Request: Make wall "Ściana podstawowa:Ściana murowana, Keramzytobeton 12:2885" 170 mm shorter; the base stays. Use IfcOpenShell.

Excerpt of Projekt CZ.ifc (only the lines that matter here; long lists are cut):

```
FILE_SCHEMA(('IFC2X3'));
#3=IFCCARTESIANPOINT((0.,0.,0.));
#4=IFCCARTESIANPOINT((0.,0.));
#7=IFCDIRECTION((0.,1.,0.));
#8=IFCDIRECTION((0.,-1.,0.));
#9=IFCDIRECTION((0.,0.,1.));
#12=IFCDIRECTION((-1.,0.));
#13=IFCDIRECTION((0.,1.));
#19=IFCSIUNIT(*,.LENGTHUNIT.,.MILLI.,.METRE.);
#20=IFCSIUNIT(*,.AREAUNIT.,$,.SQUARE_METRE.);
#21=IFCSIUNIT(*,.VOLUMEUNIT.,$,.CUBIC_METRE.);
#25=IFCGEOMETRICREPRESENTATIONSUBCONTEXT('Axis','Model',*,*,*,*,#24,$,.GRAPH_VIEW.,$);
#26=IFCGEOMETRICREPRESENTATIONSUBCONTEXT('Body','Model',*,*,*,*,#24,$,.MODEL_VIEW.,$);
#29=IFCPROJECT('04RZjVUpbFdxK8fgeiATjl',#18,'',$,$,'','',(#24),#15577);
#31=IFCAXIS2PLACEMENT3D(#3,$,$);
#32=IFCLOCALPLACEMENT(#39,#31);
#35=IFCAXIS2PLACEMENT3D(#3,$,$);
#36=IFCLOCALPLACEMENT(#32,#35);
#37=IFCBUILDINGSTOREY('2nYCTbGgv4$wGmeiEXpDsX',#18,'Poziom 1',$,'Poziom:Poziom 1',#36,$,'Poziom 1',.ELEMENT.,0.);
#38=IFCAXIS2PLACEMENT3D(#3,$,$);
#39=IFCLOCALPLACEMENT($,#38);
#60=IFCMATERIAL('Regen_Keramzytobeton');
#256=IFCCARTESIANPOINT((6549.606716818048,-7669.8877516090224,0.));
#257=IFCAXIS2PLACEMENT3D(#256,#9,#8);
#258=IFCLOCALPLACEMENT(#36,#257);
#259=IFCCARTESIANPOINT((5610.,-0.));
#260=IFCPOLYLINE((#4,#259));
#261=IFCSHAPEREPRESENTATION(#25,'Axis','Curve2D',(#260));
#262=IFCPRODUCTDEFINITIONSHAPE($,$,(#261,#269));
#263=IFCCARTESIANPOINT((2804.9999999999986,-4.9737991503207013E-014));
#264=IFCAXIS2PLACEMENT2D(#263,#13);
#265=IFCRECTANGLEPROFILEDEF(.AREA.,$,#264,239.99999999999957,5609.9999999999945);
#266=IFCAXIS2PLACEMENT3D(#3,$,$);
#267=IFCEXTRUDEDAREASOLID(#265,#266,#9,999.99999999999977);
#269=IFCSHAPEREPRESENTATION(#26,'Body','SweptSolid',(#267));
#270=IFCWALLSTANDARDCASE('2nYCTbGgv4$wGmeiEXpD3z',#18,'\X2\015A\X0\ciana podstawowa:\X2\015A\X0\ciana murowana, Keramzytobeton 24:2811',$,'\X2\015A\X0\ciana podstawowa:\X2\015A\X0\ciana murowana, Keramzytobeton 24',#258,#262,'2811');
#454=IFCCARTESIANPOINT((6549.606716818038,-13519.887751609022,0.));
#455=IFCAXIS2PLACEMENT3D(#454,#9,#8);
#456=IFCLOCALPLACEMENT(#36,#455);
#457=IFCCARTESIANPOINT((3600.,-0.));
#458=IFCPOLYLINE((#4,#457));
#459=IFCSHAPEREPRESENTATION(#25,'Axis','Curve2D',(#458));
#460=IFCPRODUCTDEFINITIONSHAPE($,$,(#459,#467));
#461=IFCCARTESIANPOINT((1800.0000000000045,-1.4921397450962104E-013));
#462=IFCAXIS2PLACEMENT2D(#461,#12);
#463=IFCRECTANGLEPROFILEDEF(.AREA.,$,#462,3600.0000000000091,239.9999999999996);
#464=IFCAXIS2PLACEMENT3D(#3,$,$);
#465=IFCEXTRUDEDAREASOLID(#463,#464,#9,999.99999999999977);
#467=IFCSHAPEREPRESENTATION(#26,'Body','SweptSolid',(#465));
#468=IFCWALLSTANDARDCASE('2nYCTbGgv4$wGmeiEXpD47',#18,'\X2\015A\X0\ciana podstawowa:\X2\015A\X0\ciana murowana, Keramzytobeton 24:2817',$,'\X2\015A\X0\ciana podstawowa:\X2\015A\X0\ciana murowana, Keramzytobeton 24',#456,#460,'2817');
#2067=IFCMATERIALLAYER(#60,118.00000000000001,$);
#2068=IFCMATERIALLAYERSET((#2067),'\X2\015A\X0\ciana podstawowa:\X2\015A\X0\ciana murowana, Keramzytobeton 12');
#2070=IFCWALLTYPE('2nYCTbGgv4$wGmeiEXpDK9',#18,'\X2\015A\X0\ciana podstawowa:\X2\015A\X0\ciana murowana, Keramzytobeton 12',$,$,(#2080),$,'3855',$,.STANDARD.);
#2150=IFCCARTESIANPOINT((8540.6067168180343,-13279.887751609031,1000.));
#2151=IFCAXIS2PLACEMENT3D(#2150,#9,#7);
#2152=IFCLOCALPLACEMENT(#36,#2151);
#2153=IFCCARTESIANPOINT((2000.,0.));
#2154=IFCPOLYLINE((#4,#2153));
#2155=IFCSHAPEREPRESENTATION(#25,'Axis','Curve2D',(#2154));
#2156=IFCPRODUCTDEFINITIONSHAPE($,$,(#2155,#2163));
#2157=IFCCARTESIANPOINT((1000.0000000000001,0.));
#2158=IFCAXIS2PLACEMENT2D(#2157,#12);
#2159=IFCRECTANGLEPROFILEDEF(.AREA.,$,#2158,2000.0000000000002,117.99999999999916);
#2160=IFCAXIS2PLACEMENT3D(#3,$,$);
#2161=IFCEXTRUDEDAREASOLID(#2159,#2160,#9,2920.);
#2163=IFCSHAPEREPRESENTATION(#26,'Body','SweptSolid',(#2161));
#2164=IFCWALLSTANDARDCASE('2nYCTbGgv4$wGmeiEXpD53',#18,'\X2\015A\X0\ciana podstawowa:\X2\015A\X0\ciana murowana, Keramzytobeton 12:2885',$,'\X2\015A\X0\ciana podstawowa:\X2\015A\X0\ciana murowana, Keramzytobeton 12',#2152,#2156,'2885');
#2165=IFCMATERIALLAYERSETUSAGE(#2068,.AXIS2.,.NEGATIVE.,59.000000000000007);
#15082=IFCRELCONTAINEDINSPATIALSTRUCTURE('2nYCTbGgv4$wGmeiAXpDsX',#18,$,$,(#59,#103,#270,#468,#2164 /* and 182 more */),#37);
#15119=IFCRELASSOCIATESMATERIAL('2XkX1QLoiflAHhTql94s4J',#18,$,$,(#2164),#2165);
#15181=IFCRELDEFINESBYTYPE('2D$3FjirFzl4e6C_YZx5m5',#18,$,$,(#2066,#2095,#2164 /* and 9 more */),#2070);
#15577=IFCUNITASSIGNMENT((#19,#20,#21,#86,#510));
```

```python
import ifcopenshell
import ifcopenshell.geom
import ifcopenshell.util.representation
import ifcopenshell.util.shape
import ifcopenshell.util.unit

model = ifcopenshell.open("Projekt CZ.ifc")
unit_scale = ifcopenshell.util.unit.calculate_unit_scale(model)
settings = ifcopenshell.geom.settings()


def volume(element):
    """Net volume in cubic metres, openings subtracted."""
    shape = ifcopenshell.geom.create_shape(settings, element)
    return ifcopenshell.util.shape.get_volume(shape.geometry)


wall = model.by_guid("2nYCTbGgv4$wGmeiEXpD53")
before = volume(wall)

body = ifcopenshell.util.representation.get_representation(wall, "Model", "Body")
solid = body.Items[0]
old_height = solid.Depth
solid.Depth -= 0.17 / unit_scale
after = volume(wall)

print(f"height {old_height:g} -> {solid.Depth:g}, volume {before:.3f} -> {after:.3f} m3")

model.write("Projekt CZ_rev.ifc")
```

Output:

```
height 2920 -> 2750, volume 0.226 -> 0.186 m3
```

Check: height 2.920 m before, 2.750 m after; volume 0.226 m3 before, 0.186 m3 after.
